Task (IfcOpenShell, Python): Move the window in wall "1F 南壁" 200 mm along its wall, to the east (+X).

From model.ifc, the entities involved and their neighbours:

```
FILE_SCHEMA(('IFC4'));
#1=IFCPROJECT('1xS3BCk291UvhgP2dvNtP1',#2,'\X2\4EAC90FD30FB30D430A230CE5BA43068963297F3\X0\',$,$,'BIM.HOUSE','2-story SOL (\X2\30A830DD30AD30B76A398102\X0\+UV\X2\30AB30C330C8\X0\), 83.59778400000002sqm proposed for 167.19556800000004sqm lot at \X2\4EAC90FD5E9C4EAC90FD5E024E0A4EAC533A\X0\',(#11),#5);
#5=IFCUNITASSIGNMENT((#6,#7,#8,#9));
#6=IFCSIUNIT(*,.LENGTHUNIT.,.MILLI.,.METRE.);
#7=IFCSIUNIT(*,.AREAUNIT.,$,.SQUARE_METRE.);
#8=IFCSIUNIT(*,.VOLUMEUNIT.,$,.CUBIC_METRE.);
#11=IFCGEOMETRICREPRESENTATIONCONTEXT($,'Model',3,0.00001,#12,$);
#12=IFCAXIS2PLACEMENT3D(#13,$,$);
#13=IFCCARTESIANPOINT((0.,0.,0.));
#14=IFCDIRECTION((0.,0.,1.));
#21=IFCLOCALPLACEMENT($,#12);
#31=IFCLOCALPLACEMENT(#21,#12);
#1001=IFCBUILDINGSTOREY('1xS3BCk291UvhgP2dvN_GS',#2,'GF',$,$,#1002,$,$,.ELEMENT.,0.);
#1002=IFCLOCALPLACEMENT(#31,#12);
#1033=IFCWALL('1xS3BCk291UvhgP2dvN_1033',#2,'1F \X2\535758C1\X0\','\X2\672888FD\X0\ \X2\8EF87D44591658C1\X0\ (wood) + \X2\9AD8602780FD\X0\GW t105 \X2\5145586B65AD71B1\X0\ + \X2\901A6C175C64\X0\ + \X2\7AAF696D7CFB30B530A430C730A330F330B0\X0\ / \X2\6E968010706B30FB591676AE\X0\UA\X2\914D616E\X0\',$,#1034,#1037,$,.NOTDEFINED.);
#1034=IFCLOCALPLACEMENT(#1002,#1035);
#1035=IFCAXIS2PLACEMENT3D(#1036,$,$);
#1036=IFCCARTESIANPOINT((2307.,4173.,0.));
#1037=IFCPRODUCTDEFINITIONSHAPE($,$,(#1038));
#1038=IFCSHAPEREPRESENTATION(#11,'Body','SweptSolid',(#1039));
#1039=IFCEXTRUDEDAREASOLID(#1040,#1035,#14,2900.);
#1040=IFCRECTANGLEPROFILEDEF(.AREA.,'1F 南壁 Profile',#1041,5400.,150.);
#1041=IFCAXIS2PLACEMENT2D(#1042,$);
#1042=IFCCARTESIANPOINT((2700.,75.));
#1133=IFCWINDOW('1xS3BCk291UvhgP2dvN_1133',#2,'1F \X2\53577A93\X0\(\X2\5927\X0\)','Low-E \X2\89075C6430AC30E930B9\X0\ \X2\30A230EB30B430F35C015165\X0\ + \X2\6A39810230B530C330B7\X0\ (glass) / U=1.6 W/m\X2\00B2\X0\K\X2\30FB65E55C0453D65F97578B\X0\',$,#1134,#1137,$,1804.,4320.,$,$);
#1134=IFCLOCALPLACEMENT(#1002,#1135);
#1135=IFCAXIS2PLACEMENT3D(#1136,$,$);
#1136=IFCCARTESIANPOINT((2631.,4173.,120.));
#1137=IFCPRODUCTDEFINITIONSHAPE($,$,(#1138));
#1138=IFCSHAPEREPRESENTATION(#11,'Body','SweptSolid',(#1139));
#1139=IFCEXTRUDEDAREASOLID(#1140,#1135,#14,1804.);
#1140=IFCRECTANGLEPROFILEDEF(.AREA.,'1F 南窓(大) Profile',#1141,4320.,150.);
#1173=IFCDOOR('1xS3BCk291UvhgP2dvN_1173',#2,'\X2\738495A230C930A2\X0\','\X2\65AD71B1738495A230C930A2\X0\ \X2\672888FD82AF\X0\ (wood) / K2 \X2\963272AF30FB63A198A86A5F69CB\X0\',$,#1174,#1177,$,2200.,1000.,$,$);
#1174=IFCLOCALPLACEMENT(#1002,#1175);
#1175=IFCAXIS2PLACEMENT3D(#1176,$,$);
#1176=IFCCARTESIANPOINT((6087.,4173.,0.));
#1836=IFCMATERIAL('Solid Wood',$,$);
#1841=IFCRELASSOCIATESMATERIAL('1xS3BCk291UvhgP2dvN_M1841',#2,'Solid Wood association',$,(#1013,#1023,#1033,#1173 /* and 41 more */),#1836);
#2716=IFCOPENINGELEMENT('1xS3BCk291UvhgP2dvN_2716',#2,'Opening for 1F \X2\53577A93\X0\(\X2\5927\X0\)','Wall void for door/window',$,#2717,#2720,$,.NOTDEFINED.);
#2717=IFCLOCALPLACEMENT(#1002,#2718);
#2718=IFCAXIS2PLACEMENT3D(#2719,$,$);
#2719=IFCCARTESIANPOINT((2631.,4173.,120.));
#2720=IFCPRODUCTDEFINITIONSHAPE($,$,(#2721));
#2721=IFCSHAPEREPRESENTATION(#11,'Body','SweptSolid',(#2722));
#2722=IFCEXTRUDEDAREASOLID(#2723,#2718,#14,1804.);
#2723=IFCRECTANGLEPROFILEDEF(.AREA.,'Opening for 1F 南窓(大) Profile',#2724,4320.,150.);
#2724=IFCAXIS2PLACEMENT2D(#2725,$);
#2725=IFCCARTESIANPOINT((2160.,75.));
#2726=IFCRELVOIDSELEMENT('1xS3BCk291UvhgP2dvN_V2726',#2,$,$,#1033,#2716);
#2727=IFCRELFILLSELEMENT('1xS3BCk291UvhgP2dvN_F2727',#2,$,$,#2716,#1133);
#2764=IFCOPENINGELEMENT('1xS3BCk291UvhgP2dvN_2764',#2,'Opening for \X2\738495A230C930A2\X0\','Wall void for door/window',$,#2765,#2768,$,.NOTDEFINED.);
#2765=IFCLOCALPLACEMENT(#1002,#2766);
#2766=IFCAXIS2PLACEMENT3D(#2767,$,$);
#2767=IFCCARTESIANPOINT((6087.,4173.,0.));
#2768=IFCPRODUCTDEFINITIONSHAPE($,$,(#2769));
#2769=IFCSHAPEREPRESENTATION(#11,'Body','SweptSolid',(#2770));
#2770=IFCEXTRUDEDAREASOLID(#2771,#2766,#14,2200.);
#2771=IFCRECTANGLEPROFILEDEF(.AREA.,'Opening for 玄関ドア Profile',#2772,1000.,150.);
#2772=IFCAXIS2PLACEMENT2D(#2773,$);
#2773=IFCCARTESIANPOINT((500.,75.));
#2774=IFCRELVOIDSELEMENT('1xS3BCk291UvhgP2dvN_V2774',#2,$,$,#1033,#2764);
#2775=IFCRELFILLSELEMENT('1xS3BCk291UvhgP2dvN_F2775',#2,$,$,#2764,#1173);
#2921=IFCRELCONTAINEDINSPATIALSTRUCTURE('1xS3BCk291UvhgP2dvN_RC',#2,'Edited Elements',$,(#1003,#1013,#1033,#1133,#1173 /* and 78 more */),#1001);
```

```python
import ifcopenshell
import ifcopenshell.api.geometry
import ifcopenshell.util.placement
import ifcopenshell.util.unit

model = ifcopenshell.open("model.ifc")
unit_scale = ifcopenshell.util.unit.calculate_unit_scale(model)

window = model.by_id(1133)
opening = window.FillsVoids[0].RelatingOpeningElement
wall = opening.VoidsElements[0].RelatingBuildingElement

wall_matrix = ifcopenshell.util.placement.get_local_placement(wall.ObjectPlacement)
shift = wall_matrix[:3, 0] * 0.2 / unit_scale
before = ifcopenshell.util.placement.get_local_placement(window.ObjectPlacement)[:3, 3].copy()

# The window is not placed relative to its opening, so move both.
for product in (opening, window):
    matrix = ifcopenshell.util.placement.get_local_placement(product.ObjectPlacement)
    matrix[:3, 3] += shift
    ifcopenshell.api.geometry.edit_object_placement(model, product=product, matrix=matrix, is_si=False)

after = ifcopenshell.util.placement.get_local_placement(window.ObjectPlacement)[:3, 3]
print("window moved by", (after - before).round(3) + 0.0)

model.write("model_updated.ifc")
```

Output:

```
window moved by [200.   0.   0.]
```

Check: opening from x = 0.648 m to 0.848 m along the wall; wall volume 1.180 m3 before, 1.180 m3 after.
